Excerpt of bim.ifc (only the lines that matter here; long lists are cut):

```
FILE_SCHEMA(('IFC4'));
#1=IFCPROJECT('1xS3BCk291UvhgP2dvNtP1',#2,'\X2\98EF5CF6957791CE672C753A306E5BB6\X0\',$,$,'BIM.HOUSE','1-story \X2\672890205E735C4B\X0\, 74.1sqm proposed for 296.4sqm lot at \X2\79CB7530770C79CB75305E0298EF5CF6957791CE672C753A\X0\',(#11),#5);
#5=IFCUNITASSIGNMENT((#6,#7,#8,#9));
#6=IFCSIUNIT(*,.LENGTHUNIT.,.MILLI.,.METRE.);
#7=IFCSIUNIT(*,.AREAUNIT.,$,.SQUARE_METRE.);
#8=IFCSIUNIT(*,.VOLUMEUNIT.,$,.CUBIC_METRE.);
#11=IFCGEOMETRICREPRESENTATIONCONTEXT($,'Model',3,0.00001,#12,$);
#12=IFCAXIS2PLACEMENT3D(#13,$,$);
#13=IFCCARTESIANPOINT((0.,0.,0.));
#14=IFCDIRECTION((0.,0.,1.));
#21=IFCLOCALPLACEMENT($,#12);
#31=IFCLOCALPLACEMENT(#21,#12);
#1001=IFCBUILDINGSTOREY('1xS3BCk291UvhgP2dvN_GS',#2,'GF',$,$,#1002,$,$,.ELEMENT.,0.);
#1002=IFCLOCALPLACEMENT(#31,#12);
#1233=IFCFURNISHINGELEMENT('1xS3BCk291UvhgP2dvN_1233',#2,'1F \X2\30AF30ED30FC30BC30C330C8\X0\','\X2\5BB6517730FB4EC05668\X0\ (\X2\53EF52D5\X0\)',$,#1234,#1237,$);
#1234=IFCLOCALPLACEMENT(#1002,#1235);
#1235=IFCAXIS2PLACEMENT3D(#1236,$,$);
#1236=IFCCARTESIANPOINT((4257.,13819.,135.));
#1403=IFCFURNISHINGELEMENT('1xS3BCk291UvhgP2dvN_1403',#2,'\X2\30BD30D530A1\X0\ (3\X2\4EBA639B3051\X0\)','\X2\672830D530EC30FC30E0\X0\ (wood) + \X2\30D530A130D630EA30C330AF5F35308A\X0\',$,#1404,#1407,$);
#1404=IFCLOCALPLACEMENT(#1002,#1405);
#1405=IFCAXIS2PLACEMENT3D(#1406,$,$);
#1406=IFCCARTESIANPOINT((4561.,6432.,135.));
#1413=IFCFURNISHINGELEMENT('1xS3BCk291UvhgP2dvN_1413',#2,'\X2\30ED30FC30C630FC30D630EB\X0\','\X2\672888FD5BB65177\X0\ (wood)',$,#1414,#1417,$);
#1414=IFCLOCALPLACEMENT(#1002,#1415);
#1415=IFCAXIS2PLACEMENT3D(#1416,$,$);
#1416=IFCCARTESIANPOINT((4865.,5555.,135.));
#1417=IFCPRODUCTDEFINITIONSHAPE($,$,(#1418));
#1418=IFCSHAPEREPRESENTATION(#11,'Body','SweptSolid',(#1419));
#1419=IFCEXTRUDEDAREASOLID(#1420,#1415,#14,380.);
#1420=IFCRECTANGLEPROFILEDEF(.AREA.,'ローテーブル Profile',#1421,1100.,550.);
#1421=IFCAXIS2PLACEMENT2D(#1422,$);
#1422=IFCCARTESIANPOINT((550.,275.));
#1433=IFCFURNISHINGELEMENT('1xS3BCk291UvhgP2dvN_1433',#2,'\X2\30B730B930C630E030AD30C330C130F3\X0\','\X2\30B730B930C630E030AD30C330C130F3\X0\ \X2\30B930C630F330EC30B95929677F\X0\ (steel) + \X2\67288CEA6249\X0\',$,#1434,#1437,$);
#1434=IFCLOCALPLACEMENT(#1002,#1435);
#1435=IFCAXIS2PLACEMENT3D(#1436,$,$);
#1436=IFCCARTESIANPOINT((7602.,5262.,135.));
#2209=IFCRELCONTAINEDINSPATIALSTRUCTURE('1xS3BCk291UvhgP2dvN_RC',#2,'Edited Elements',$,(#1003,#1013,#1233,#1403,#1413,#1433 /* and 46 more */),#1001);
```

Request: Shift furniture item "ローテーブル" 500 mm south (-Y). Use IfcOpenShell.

```python
import ifcopenshell
import ifcopenshell.api.geometry
import ifcopenshell.util.placement
import ifcopenshell.util.unit

model = ifcopenshell.open("bim.ifc")
unit_scale = ifcopenshell.util.unit.calculate_unit_scale(model)

item = model.by_id(1413)
matrix = ifcopenshell.util.placement.get_local_placement(item.ObjectPlacement)
matrix[1, 3] -= 0.5 / unit_scale
ifcopenshell.api.geometry.edit_object_placement(model, product=item, matrix=matrix, is_si=False)

print(ifcopenshell.util.placement.get_local_placement(item.ObjectPlacement).round(3) + 0.0)

model.write("bim_updated.ifc")
```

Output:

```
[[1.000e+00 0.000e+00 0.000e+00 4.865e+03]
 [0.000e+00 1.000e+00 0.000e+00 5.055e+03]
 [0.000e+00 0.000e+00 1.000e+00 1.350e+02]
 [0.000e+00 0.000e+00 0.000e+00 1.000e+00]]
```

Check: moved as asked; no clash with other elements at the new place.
